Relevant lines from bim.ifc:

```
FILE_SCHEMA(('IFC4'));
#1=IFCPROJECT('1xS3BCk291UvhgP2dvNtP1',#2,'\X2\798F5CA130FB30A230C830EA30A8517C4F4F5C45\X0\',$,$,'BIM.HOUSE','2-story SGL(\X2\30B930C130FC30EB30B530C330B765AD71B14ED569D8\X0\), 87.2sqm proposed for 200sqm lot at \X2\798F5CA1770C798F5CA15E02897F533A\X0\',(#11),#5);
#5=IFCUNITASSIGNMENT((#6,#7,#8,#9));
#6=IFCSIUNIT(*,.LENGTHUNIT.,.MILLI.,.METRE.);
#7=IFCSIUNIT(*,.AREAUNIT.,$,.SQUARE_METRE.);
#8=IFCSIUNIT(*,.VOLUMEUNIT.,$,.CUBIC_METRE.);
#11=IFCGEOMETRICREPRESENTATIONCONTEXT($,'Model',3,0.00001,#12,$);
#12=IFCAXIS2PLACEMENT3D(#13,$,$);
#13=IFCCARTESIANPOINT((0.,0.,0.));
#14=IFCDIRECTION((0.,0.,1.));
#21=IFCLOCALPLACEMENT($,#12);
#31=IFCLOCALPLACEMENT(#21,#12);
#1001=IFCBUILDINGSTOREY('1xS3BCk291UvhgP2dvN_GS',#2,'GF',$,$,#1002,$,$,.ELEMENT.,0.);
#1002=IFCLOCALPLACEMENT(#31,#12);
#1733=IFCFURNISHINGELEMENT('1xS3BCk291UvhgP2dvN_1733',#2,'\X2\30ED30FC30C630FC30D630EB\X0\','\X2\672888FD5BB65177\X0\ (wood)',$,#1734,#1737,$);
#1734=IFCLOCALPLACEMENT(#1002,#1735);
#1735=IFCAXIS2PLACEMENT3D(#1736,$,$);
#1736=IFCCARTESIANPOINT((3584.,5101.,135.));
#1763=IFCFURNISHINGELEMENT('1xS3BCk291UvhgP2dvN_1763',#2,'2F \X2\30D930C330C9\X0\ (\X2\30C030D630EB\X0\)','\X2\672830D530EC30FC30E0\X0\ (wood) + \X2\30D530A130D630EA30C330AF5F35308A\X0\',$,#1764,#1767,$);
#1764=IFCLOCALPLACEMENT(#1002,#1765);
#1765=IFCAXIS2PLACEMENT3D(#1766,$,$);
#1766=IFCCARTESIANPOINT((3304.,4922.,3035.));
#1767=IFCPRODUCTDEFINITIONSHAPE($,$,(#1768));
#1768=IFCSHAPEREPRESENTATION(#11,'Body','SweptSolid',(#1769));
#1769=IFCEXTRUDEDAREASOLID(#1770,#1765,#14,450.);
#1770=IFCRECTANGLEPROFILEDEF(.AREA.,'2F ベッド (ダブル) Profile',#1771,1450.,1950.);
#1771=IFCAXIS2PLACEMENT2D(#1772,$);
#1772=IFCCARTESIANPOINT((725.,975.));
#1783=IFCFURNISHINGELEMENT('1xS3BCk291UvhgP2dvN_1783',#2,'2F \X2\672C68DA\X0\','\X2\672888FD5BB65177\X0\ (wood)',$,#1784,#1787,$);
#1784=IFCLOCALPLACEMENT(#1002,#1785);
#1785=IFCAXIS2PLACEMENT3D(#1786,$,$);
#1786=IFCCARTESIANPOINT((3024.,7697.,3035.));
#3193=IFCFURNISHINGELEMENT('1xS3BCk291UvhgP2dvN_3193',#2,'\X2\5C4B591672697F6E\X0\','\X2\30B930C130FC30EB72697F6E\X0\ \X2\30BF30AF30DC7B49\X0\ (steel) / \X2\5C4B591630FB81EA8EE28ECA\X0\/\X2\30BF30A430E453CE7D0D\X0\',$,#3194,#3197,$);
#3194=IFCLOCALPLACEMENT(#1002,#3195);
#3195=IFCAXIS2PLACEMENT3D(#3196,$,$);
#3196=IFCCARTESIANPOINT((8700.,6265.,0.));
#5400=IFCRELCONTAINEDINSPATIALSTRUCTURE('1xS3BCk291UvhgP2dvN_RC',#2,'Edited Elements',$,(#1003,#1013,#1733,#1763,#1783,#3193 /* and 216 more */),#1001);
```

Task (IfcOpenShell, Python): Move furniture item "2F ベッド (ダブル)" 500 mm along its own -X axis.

```python
import ifcopenshell
import ifcopenshell.api.geometry
import ifcopenshell.util.placement
import ifcopenshell.util.unit

model = ifcopenshell.open("bim.ifc")
unit_scale = ifcopenshell.util.unit.calculate_unit_scale(model)

item = model.by_id(1763)
matrix = ifcopenshell.util.placement.get_local_placement(item.ObjectPlacement)
matrix[:3, 3] -= matrix[:3, 0] * 0.5 / unit_scale
ifcopenshell.api.geometry.edit_object_placement(model, product=item, matrix=matrix, is_si=False)

print(ifcopenshell.util.placement.get_local_placement(item.ObjectPlacement).round(3) + 0.0)

model.write("bim_rev.ifc")
```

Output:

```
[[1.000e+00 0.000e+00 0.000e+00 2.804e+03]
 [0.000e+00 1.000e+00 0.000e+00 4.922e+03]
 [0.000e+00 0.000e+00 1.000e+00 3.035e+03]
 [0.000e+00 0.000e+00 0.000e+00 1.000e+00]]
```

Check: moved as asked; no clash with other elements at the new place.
